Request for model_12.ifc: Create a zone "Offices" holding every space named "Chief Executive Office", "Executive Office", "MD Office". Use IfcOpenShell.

First a look at what the model holds.

```python
import ifcopenshell

model = ifcopenshell.open("model_12.ifc")
print(model.schema)
seen = {}
for space in model.by_type("IfcSpace"):
    seen[space.LongName] = seen.get(space.LongName, 0) + 1
for name, count in sorted(seen.items(), key=str):
    print(count, "x", name)
print("zones:", [z.Name for z in model.by_type("IfcZone")][:20])
```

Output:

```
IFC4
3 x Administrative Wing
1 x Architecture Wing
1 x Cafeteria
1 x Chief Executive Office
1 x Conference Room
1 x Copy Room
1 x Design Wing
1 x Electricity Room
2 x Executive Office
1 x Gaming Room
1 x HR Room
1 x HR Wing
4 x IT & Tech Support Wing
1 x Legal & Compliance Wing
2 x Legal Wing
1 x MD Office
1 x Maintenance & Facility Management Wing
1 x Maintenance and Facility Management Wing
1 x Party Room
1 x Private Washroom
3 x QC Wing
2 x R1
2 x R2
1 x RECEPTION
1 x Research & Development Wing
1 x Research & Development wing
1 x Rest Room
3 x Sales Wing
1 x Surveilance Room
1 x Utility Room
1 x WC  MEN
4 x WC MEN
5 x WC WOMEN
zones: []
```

```python
import ifcopenshell
import ifcopenshell.api.group
import ifcopenshell.api.root

model = ifcopenshell.open("model_12.ifc")

names = {"Chief Executive Office", "Executive Office", "MD Office"}
spaces = [s for s in model.by_type("IfcSpace") if s.LongName in names]

zone = ifcopenshell.api.root.create_entity(model, ifc_class="IfcZone", name="Offices")
ifcopenshell.api.group.assign_group(model, products=spaces, group=zone)
print(len(spaces), "spaces in", zone.Name)

model.write("model_12_updated.ifc")
```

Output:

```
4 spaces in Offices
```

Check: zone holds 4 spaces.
